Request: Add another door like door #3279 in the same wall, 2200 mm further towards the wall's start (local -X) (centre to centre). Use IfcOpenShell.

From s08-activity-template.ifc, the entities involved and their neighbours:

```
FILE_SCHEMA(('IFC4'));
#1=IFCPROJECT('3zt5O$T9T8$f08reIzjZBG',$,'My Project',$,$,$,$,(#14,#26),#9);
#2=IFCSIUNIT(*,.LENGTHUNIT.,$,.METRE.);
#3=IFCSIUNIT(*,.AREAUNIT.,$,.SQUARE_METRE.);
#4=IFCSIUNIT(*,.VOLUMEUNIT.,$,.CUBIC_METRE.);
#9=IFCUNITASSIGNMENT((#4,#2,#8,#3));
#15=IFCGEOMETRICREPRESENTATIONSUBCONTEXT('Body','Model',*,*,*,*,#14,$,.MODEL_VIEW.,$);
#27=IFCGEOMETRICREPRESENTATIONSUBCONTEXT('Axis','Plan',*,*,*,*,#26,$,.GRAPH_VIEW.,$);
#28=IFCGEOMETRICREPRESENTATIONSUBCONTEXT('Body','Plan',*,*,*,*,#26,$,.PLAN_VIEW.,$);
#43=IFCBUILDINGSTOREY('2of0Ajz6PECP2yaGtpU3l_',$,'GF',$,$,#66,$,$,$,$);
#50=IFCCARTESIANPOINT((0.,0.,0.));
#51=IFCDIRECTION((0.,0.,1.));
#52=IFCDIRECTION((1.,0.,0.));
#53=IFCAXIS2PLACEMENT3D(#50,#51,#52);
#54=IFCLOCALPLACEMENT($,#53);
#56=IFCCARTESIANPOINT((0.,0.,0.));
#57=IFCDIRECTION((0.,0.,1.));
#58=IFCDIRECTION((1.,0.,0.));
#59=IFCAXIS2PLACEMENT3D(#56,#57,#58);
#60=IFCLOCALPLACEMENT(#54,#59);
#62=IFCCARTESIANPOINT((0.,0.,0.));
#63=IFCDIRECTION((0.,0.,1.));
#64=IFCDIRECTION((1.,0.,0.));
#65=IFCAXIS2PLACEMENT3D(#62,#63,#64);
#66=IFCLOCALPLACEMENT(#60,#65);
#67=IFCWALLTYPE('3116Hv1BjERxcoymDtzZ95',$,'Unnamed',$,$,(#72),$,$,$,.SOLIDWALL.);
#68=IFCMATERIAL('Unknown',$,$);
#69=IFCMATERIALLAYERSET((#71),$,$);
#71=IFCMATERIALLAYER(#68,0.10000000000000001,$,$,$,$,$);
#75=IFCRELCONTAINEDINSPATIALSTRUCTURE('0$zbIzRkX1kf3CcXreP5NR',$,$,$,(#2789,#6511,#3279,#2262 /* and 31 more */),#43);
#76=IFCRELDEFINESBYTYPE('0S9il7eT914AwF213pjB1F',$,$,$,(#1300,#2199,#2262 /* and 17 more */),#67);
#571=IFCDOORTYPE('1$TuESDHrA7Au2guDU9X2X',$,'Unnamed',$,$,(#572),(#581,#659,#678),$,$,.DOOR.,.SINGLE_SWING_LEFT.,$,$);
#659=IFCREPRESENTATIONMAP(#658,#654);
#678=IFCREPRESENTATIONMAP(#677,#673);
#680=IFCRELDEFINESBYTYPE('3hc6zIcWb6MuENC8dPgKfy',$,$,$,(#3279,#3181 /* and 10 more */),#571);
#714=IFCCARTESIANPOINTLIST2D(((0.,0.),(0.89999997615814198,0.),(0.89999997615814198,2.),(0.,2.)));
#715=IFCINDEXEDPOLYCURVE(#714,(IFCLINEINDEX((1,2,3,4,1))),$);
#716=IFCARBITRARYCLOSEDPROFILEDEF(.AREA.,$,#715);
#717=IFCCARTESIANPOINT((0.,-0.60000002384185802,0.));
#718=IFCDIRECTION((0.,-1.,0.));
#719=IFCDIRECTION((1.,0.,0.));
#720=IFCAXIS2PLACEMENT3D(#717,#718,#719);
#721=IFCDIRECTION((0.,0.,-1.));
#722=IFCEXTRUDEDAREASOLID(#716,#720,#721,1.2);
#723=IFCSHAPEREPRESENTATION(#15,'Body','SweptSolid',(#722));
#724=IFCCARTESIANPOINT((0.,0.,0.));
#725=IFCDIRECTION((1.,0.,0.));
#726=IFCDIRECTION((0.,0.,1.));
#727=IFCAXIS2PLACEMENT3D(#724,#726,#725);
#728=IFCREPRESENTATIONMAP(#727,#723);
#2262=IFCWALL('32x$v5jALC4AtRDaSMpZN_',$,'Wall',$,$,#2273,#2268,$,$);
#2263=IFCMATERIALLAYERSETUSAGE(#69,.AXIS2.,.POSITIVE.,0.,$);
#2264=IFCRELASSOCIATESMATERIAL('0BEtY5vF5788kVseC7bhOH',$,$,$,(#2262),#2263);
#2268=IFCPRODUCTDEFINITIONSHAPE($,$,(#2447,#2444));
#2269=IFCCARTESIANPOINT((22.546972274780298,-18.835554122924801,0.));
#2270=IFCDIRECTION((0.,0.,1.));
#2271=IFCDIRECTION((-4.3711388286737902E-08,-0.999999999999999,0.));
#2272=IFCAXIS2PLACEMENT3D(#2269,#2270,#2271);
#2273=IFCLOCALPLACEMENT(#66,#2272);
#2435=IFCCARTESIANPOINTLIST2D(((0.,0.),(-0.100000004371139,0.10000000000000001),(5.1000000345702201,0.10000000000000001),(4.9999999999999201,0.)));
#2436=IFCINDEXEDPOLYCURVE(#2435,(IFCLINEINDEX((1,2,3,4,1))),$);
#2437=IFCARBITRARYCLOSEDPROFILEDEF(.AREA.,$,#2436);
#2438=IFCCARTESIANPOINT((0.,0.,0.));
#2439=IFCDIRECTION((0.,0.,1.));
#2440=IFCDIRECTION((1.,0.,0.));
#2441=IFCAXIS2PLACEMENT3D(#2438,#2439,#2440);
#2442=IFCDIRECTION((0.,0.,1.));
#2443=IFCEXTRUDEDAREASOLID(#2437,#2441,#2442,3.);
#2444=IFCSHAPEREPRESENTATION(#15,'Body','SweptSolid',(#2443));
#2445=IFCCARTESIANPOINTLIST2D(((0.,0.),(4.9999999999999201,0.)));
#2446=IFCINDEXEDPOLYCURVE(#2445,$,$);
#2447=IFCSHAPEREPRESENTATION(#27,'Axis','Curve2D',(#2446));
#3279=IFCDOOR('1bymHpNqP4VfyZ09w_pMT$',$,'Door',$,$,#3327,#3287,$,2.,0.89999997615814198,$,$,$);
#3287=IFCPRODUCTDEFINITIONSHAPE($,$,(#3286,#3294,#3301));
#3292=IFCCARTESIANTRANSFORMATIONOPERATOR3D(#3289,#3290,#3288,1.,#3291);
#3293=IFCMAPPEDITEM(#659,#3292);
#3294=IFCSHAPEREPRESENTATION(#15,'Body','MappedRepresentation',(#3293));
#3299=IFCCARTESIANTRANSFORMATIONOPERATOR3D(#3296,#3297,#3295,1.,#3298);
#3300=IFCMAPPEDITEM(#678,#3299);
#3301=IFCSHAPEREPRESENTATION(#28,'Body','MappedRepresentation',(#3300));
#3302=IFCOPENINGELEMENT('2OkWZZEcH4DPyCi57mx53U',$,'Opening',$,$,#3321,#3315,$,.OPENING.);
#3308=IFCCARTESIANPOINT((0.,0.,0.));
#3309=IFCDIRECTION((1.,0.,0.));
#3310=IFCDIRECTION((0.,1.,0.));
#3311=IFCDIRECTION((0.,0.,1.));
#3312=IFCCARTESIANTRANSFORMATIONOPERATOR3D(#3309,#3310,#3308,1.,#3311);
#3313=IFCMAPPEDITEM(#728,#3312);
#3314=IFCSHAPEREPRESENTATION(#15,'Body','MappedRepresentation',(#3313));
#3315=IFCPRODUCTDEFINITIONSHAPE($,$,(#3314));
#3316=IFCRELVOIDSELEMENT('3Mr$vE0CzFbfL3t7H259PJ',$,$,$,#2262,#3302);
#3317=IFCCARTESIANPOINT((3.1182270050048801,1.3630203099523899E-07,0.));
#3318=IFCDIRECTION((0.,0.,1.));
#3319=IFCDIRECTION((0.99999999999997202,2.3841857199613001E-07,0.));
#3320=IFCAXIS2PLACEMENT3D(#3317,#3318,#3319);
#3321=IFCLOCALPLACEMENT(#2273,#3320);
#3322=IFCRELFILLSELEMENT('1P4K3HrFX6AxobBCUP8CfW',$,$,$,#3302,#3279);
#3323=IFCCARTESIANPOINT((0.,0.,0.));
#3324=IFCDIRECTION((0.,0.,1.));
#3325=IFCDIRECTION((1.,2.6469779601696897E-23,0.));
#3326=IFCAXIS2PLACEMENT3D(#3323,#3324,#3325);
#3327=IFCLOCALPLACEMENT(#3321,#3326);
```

```python
import ifcopenshell
import ifcopenshell.api.feature
import ifcopenshell.api.geometry
import ifcopenshell.api.root
import ifcopenshell.geom
import ifcopenshell.util.element
import ifcopenshell.util.placement
import ifcopenshell.util.shape
import ifcopenshell.util.unit

model = ifcopenshell.open("s08-activity-template.ifc")
unit_scale = ifcopenshell.util.unit.calculate_unit_scale(model)
settings = ifcopenshell.geom.settings()


def volume(element):
    """Net volume in cubic metres, openings subtracted."""
    shape = ifcopenshell.geom.create_shape(settings, element)
    return ifcopenshell.util.shape.get_volume(shape.geometry)


door = model.by_guid("1bymHpNqP4VfyZ09w_pMT$")
opening = door.FillsVoids[0].RelatingOpeningElement
wall = opening.VoidsElements[0].RelatingBuildingElement
before = volume(wall)
shift = ifcopenshell.util.placement.get_local_placement(wall.ObjectPlacement)[:3, 0] * -2.2 / unit_scale

# copy_class copies the void relationship, type, container and properties, but no geometry.
new_opening = ifcopenshell.api.root.copy_class(model, product=opening)
new_opening.Representation = ifcopenshell.util.element.copy_deep(
    model, opening.Representation, exclude=["IfcGeometricRepresentationContext", "IfcRepresentationMap"]
)
new_door = ifcopenshell.api.root.copy_class(model, product=door)
new_door.Representation = ifcopenshell.util.element.copy_deep(
    model, door.Representation, exclude=["IfcGeometricRepresentationContext", "IfcRepresentationMap"]
)
ifcopenshell.api.feature.add_filling(model, opening=new_opening, element=new_door)

for old, new in ((opening, new_opening), (door, new_door)):
    matrix = ifcopenshell.util.placement.get_local_placement(old.ObjectPlacement)
    matrix[:3, 3] += shift
    ifcopenshell.api.geometry.edit_object_placement(model, product=new, matrix=matrix, is_si=False)

after = volume(wall)

print(f"wall volume {before:.3f} -> {after:.3f} m3")

model.write("s08-activity-template_v2.ifc")
```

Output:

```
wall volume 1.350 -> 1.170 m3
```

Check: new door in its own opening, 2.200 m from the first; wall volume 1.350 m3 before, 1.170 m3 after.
